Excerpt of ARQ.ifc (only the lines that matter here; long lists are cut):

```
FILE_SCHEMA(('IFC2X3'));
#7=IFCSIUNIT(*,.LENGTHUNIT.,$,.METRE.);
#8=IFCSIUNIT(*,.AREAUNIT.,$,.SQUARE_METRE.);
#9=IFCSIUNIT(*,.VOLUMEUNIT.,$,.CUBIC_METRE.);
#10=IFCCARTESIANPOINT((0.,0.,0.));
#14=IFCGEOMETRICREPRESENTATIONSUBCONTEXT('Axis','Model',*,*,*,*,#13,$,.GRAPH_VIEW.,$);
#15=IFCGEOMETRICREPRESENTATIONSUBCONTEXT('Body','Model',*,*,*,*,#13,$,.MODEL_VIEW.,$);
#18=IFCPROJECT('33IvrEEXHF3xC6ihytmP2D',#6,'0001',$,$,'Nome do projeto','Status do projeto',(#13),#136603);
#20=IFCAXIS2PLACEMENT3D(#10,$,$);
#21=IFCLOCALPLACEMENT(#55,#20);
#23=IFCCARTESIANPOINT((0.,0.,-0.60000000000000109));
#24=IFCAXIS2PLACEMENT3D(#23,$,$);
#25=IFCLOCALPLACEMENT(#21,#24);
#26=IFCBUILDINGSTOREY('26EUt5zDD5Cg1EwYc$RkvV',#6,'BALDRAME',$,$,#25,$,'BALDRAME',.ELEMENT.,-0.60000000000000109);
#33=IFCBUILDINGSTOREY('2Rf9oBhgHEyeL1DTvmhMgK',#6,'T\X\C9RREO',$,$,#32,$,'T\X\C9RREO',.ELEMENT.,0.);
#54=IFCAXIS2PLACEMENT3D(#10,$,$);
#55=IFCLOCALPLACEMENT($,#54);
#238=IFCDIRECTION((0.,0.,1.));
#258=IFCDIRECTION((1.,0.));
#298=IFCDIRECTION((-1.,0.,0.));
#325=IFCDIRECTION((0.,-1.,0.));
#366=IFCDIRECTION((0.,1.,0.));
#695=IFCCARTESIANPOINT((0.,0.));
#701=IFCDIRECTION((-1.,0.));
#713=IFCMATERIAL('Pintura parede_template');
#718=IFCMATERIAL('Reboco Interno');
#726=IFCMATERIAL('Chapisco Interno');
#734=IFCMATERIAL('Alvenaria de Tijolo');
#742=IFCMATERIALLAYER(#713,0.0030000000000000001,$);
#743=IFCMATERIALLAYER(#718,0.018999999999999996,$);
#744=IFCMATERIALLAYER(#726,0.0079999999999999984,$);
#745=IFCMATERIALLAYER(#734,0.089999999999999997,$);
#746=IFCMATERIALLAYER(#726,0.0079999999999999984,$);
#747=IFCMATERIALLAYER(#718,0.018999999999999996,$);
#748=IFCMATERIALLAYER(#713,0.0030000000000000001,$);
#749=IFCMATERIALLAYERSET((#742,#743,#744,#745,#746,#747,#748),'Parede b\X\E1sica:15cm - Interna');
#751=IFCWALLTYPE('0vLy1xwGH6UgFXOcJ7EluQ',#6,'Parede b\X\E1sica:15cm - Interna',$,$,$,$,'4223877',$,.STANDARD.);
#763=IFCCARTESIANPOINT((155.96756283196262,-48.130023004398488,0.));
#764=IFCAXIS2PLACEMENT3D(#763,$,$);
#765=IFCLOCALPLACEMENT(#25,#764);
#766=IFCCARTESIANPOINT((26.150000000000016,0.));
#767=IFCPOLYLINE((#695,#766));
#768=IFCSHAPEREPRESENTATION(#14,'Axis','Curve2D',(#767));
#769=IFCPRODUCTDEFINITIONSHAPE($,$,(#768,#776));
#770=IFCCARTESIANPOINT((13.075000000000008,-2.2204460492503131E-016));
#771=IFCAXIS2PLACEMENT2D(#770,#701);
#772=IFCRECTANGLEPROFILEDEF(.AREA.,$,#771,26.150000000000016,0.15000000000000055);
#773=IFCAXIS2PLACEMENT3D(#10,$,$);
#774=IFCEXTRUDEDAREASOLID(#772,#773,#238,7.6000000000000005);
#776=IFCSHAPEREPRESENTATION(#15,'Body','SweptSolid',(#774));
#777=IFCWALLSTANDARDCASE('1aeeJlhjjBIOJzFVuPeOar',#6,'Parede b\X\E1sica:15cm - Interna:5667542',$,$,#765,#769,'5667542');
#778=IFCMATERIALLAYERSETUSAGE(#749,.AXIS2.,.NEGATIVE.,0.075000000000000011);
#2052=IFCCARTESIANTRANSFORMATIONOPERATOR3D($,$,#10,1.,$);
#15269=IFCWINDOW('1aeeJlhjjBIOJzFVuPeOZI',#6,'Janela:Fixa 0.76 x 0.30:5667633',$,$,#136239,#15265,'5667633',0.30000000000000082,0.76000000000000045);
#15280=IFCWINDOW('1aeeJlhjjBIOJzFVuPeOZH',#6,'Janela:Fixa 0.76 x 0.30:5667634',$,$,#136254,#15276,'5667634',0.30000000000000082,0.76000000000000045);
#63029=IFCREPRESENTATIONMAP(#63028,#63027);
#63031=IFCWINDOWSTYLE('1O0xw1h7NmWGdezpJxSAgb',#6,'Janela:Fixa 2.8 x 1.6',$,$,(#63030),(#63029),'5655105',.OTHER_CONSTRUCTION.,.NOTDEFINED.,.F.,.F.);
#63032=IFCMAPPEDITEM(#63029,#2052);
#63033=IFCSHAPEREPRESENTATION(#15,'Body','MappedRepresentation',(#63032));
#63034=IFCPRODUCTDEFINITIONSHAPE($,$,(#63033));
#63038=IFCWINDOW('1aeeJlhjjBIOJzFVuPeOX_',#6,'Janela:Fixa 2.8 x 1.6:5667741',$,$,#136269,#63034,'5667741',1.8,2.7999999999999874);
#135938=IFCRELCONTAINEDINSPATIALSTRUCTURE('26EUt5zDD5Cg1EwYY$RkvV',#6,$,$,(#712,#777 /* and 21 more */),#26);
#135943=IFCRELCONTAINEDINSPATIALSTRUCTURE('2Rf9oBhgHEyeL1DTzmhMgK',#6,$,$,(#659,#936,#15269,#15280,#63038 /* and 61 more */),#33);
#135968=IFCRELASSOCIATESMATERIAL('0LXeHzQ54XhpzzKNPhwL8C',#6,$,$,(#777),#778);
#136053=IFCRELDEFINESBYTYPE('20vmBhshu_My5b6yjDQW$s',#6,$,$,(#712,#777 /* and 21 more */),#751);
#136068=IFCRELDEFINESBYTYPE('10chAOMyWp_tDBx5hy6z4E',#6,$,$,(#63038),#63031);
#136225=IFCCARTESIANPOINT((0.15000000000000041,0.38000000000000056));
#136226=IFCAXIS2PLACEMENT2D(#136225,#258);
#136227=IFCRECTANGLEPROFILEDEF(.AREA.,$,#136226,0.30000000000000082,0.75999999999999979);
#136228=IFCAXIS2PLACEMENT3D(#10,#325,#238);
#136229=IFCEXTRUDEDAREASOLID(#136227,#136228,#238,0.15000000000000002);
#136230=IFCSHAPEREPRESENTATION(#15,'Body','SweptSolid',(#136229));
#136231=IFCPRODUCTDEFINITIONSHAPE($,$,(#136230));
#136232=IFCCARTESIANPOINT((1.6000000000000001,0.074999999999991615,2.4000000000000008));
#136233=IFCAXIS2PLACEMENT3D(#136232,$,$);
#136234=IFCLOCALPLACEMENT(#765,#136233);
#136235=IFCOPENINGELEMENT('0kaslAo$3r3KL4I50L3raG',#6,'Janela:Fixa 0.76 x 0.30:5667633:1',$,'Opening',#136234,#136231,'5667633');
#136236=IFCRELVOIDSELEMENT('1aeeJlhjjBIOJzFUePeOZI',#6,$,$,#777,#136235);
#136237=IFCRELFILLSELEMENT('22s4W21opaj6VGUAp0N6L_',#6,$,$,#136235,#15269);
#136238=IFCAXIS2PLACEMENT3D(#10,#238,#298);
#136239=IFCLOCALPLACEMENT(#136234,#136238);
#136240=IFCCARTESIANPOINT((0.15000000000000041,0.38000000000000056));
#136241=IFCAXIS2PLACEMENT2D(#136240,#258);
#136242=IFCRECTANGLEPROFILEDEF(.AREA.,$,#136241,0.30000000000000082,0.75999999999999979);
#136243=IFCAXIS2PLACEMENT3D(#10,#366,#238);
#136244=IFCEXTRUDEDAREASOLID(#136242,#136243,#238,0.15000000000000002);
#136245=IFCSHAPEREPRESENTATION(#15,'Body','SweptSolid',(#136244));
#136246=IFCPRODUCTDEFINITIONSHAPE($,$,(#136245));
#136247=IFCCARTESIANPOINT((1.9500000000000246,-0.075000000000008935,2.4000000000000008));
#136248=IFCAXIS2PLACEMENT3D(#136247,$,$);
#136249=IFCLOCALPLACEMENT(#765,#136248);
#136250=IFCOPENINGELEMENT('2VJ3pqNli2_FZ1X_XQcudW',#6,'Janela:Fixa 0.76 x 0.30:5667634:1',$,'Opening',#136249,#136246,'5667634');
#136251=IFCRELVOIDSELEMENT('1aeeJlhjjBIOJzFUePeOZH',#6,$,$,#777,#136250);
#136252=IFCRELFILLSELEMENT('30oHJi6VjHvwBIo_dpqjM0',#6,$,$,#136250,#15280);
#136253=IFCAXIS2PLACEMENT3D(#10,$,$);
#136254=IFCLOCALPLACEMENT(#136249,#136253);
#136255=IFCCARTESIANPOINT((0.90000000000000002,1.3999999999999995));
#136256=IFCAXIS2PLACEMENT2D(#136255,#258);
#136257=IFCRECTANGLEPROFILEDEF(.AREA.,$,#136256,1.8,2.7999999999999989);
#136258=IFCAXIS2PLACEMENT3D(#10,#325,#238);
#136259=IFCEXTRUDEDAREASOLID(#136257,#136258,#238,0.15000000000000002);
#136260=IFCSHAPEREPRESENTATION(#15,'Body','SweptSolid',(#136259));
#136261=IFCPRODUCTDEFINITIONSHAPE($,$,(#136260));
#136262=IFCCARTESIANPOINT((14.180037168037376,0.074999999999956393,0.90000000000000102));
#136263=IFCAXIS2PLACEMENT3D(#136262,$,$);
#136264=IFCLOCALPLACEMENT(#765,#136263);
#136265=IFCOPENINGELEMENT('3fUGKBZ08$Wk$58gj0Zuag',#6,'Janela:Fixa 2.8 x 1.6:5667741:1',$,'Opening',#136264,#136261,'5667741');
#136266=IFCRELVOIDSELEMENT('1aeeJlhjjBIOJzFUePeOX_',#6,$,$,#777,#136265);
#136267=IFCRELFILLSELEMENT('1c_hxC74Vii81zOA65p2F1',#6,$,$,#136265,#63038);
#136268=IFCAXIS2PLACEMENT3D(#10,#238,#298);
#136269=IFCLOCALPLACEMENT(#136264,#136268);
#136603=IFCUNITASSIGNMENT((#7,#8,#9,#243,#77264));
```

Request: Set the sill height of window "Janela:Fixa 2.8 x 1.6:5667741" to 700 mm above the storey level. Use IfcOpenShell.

```python
import numpy as np
import ifcopenshell
import ifcopenshell.api.geometry
import ifcopenshell.geom
import ifcopenshell.util.element
import ifcopenshell.util.placement
import ifcopenshell.util.shape
import ifcopenshell.util.unit

model = ifcopenshell.open("ARQ.ifc")
unit_scale = ifcopenshell.util.unit.calculate_unit_scale(model)

window = model.by_guid("1aeeJlhjjBIOJzFVuPeOX_")
opening = window.FillsVoids[0].RelatingOpeningElement
storey = ifcopenshell.util.element.get_container(window, ifc_class="IfcBuildingStorey")
level = ifcopenshell.util.placement.get_local_placement(storey.ObjectPlacement)[2, 3]

# The opening's origin need not be at the sill, so measure its lowest point.
shape = ifcopenshell.geom.create_shape(ifcopenshell.geom.settings(), opening)
bottom = ifcopenshell.util.shape.get_shape_bottom_elevation(shape, shape.geometry) / unit_scale
dz = level + 0.7 / unit_scale - bottom

shift = np.array([0.0, 0.0, dz])
# The window is placed relative to its opening, so it follows when the opening moves.
matrix = ifcopenshell.util.placement.get_local_placement(opening.ObjectPlacement)
matrix[:3, 3] += shift
ifcopenshell.api.geometry.edit_object_placement(
    model, product=opening, matrix=matrix, is_si=False, should_transform_children=True
)

print(f"moved by {dz * unit_scale:+.3f} m")

model.write("ARQ_updated.ifc")
```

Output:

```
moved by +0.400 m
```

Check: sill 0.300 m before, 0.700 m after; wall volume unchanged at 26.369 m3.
